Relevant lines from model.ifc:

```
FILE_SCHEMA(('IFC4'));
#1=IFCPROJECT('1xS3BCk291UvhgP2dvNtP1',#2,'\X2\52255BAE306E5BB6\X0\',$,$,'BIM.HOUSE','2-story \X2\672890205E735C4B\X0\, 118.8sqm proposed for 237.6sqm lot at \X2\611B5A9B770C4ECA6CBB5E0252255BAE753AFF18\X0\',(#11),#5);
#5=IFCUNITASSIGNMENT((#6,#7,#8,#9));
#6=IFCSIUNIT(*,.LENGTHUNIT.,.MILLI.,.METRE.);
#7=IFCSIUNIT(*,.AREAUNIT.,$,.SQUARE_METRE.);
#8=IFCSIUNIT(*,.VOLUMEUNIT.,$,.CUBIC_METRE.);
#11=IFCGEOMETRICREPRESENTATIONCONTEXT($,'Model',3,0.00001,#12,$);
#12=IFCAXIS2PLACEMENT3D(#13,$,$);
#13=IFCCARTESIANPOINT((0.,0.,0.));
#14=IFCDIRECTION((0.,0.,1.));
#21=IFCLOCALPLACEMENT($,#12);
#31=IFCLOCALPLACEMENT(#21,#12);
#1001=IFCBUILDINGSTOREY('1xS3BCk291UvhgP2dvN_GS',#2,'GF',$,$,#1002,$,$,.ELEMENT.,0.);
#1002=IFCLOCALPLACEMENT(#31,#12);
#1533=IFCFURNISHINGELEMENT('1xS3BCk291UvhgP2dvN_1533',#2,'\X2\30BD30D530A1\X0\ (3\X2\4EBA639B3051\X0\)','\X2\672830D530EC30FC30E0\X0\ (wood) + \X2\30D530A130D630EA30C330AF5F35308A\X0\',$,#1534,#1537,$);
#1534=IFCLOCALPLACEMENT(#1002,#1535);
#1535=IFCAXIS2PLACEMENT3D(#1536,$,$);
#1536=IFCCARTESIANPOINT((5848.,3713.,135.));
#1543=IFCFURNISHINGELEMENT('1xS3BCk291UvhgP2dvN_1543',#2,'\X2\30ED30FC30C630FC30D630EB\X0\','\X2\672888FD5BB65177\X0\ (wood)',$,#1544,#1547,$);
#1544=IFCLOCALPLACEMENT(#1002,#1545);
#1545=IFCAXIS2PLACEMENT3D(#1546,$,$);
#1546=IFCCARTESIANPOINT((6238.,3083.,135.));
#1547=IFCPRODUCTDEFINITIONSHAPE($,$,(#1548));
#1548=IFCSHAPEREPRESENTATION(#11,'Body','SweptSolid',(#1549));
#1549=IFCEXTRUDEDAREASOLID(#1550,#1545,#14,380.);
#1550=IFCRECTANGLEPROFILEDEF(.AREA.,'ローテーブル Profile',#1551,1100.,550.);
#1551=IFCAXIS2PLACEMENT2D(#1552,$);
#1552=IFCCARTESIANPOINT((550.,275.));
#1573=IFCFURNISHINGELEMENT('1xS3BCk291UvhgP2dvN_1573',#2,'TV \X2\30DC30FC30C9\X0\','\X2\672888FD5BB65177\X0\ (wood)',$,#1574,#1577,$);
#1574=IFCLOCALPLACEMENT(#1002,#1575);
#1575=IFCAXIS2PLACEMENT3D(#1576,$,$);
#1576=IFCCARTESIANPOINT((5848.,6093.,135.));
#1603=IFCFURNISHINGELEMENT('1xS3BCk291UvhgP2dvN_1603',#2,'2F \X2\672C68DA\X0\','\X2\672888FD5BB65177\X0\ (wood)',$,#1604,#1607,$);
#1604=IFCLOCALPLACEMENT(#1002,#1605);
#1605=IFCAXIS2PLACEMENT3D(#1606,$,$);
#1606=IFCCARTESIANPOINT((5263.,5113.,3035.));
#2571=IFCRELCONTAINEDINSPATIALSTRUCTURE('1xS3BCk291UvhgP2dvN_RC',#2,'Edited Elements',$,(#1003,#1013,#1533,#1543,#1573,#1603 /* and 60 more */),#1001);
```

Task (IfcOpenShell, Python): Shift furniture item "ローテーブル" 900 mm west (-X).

```python
import ifcopenshell
import ifcopenshell.api.geometry
import ifcopenshell.util.placement

model = ifcopenshell.open("model.ifc")

item = model.by_guid("1xS3BCk291UvhgP2dvN_1543")
matrix = ifcopenshell.util.placement.get_local_placement(item.ObjectPlacement)
matrix[0, 3] -= 900.0
ifcopenshell.api.geometry.edit_object_placement(model, product=item, matrix=matrix, is_si=False)

print(ifcopenshell.util.placement.get_local_placement(item.ObjectPlacement).round(3) + 0.0)

model.write("model_edited.ifc")
```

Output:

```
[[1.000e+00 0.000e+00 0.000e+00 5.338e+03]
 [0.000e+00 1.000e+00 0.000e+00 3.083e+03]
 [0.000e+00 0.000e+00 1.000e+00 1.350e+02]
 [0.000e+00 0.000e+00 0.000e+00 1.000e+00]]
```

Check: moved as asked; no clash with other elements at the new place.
